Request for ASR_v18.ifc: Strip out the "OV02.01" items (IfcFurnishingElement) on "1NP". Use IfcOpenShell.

First a look at what the model holds.

```python
import ifcopenshell
import ifcopenshell.util.element

model = ifcopenshell.open("ASR_v18.ifc")
print(model.schema)
storey = next(s for s in model.by_type("IfcBuildingStorey") if s.Name == "1NP")
furniture = [e for e in ifcopenshell.util.element.get_decomposition(storey) if e.is_a("IfcFurnishingElement")]
seen = {}
for e in furniture:
    element_type = ifcopenshell.util.element.get_type(e)
    name = element_type.Name if element_type not in (None, e) else None
    seen[name] = seen.get(name, 0) + 1
for name, count in sorted(seen.items(), key=str):
    print(count, "x", name)
```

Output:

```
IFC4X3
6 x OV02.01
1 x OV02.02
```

```python
import ifcopenshell
import ifcopenshell.api.root
import ifcopenshell.util.element

model = ifcopenshell.open("ASR_v18.ifc")

storey = next(s for s in model.by_type("IfcBuildingStorey") if s.Name == "1NP")
furniture = [e for e in ifcopenshell.util.element.get_decomposition(storey) if e.is_a("IfcFurnishingElement")]
targets = [e for e in furniture if (t := ifcopenshell.util.element.get_type(e)) not in (None, e) and t.Name == "OV02.01"]

for e in targets:
    ifcopenshell.api.root.remove_product(model, product=e)
print(len(targets), "removed")

model.write("ASR_v18-out.ifc")
```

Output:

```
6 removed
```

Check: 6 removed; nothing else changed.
